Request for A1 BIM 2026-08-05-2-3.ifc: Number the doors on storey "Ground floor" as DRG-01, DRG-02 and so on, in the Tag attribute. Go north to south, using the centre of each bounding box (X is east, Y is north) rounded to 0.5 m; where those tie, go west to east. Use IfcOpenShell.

First a look at what the model holds.

```python
import ifcopenshell
import ifcopenshell.util.element
import ifcopenshell.util.placement

model = ifcopenshell.open("A1 BIM 2026-08-05-2-3.ifc")
print(model.schema)
storey = next(s for s in model.by_type("IfcBuildingStorey") if s.Name == "Ground floor")
doors = [e for e in ifcopenshell.util.element.get_decomposition(storey) if e.is_a("IfcDoor")]
for e in sorted(doors, key=lambda e: e.id()):
    origin = ifcopenshell.util.placement.get_local_placement(e.ObjectPlacement)[:3, 3]
    print(e.id(), e.Tag, e.Name, origin.round(2) + 0.0, sep=" | ")
```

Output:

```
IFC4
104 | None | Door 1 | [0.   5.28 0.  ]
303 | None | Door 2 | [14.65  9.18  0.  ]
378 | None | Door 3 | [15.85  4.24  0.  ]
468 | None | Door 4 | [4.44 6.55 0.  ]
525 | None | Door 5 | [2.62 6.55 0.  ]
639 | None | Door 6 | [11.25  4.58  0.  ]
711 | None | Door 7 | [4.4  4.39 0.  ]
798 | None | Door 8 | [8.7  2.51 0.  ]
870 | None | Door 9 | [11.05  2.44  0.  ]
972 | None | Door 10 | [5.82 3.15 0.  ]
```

```python
import ifcopenshell
import ifcopenshell.geom
import ifcopenshell.util.element
import ifcopenshell.util.shape

model = ifcopenshell.open("A1 BIM 2026-08-05-2-3.ifc")
settings = ifcopenshell.geom.settings()
settings.set("use-world-coords", True)


def centre(element):
    shape = ifcopenshell.geom.create_shape(settings, element)
    return ifcopenshell.util.shape.get_bbox_centroid(shape.geometry)


storey = next(s for s in model.by_type("IfcBuildingStorey") if s.Name == "Ground floor")
doors = [e for e in ifcopenshell.util.element.get_decomposition(storey) if e.is_a("IfcDoor")]

# Insertion points can sit at a corner or the storey origin, so sort by the geometry (in metres).
centres = {e: centre(e) for e in doors}
doors.sort(key=lambda e: (-round(centres[e][1] / 0.5), centres[e][0]))

for i, e in enumerate(doors, start=1):
    number = f"DRG-{i:02d}"
    e.Tag = number
    print(e.id(), number)

model.write("A1 BIM 2026-08-05-2-3_v2.ifc")
```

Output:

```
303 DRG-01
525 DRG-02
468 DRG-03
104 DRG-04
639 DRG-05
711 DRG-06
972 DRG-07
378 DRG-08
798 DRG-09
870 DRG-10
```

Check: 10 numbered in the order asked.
